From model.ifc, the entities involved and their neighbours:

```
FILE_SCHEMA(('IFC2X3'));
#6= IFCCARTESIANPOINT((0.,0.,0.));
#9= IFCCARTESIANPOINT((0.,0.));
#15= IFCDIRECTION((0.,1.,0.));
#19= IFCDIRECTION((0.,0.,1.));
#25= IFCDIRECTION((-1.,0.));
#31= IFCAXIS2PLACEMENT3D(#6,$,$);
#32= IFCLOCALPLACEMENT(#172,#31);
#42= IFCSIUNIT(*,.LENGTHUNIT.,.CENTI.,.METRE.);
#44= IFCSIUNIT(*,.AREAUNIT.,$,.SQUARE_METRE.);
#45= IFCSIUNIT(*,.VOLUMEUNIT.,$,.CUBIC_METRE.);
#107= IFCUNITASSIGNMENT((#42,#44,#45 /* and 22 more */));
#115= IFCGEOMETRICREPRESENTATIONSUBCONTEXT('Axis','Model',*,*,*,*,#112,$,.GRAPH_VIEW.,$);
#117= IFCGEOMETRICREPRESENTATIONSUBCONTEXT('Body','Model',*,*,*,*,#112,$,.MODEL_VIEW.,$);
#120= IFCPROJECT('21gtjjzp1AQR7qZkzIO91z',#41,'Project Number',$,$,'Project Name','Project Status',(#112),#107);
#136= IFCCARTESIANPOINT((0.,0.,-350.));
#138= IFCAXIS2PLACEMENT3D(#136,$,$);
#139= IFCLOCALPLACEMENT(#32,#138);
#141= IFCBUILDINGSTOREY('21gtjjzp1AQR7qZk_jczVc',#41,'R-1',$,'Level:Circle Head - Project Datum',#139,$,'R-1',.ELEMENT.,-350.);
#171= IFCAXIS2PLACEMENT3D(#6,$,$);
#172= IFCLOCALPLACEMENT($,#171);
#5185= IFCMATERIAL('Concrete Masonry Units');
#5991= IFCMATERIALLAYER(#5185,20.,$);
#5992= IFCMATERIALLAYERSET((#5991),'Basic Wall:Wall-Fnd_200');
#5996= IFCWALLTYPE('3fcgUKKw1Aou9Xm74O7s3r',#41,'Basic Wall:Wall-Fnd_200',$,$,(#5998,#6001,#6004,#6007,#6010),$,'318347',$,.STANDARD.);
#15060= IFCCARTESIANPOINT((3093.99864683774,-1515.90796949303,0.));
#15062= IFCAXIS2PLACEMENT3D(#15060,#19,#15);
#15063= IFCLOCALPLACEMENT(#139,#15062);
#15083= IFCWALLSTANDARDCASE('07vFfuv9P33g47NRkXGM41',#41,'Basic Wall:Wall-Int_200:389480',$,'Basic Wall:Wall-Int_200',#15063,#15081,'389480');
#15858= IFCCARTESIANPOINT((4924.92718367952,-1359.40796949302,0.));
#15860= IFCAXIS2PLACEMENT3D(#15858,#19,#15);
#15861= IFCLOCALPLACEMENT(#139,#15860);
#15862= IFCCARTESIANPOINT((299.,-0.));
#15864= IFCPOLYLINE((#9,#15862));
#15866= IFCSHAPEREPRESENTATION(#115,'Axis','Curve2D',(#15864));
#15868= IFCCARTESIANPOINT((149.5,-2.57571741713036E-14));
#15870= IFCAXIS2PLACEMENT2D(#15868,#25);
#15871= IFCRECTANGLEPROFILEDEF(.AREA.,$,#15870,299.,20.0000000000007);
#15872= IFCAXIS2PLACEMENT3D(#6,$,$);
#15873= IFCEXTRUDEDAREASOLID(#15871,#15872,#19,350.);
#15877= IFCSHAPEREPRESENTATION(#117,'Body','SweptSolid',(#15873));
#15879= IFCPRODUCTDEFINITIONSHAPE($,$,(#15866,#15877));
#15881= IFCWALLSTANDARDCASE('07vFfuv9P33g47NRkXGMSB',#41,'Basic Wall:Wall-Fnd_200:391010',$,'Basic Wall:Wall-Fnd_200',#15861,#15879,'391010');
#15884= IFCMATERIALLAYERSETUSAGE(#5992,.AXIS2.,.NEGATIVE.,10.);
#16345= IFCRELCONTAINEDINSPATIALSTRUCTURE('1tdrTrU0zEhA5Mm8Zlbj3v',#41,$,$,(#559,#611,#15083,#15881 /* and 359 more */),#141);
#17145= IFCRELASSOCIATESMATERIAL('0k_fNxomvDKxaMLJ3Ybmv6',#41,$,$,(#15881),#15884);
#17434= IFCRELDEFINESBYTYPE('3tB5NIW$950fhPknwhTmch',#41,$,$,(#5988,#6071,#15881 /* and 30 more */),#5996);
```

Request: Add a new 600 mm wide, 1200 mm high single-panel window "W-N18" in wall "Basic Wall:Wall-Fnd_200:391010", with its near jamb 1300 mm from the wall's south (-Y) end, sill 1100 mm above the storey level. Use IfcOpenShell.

```python
import numpy as np
import ifcopenshell
import ifcopenshell.api.feature
import ifcopenshell.api.geometry
import ifcopenshell.api.root
import ifcopenshell.api.spatial
import ifcopenshell.api.type
import ifcopenshell.geom
import ifcopenshell.util.element
import ifcopenshell.util.placement
import ifcopenshell.util.representation
import ifcopenshell.util.shape
import ifcopenshell.util.unit

model = ifcopenshell.open("model.ifc")
unit_scale = ifcopenshell.util.unit.calculate_unit_scale(model)
settings = ifcopenshell.geom.settings()


def volume(element):
    """Net volume in cubic metres, openings subtracted."""
    shape = ifcopenshell.geom.create_shape(settings, element)
    return ifcopenshell.util.shape.get_volume(shape.geometry)


wall = model.by_guid("07vFfuv9P33g47NRkXGMSB")
storey = ifcopenshell.util.element.get_container(wall, ifc_class="IfcBuildingStorey")
context = ifcopenshell.util.representation.get_context(model, "Model", "Body", "MODEL_VIEW")
before = volume(wall)

width, height, from_end, sill = 0.6, 1.2, 1.3, 1.1  # metres

# The wall runs along its own X axis, and the end named is its -X end.
wall_shape = ifcopenshell.geom.create_shape(settings, wall)
x, y, z = ifcopenshell.util.shape.get_vertices(wall_shape.geometry).T
start = x.min() + from_end
face, thickness = float(y.min()), float(y.max() - y.min())
wall_matrix = ifcopenshell.util.placement.get_local_placement(wall.ObjectPlacement)
level = ifcopenshell.util.placement.get_local_placement(storey.ObjectPlacement)[2, 3]


def in_wall(x, y):
    """Placement at x, y metres in the wall's axes, at sill height."""
    matrix = wall_matrix.copy()
    matrix[:, 3] = wall_matrix @ np.array([x / unit_scale, y / unit_scale, 0.0, 1.0])
    matrix[2, 3] = level + sill / unit_scale
    return matrix


# Opening: a box that overshoots both wall faces by 50 mm.
opening = ifcopenshell.api.root.create_entity(model, ifc_class="IfcOpeningElement")
box = ifcopenshell.api.geometry.add_wall_representation(
    model, context=context, length=width, height=height, thickness=thickness + 0.1
)
ifcopenshell.api.geometry.assign_representation(model, product=opening, representation=box)
ifcopenshell.api.geometry.edit_object_placement(model, product=opening, matrix=in_wall(start, face - 0.05), is_si=False)
ifcopenshell.api.feature.add_feature(model, feature=opening, element=wall)

window = ifcopenshell.api.root.create_entity(model, ifc_class="IfcWindow", name="W-N18")
window.OverallWidth, window.OverallHeight = width / unit_scale, height / unit_scale
body = ifcopenshell.api.geometry.add_window_representation(
    model,
    context=context,
    overall_width=window.OverallWidth,
    overall_height=window.OverallHeight,
    partition_type="SINGLE_PANEL",
)
ifcopenshell.api.geometry.assign_representation(model, product=window, representation=body)
ifcopenshell.api.spatial.assign_container(model, products=[window], relating_structure=storey)
fills = ifcopenshell.api.feature.add_filling(model, opening=opening, element=window)
fills.OwnerHistory = window.OwnerHistory  # required in IFC2X3

# IFC2X3 keeps the operation on the window style.
style = ifcopenshell.api.root.create_entity(model, ifc_class="IfcWindowStyle", name="W-N18")
style.OperationType, style.ConstructionType = "SINGLE_PANEL", "NOTDEFINED"
style.ParameterTakesPrecedence = style.Sizeable = False
ifcopenshell.api.type.assign_type(model, related_objects=[window], relating_type=style)

# Centre the window in the wall's thickness.
ifcopenshell.api.geometry.edit_object_placement(model, product=window, matrix=in_wall(start, face), is_si=False)
window_shape = ifcopenshell.geom.create_shape(settings, window)
depth = ifcopenshell.util.shape.get_vertices(window_shape.geometry)[:, 1]
offset = face + thickness / 2 - (depth.min() + depth.max()) / 2
ifcopenshell.api.geometry.edit_object_placement(model, product=window, matrix=in_wall(start, offset), is_si=False)

after = volume(wall)

print(f"wall volume {before:.3f} -> {after:.3f} m3")

model.write("model_v2.ifc")
```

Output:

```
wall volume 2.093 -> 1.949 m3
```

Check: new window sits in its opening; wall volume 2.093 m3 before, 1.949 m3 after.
